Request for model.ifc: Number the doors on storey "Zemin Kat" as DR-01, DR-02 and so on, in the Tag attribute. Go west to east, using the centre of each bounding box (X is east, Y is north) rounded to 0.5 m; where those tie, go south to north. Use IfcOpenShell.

First a look at what the model holds.

```python
import ifcopenshell
import ifcopenshell.util.element
import ifcopenshell.util.placement

model = ifcopenshell.open("model.ifc")
print(model.schema)
storey = next(s for s in model.by_type("IfcBuildingStorey") if s.Name == "Zemin Kat")
doors = [e for e in ifcopenshell.util.element.get_decomposition(storey) if e.is_a("IfcDoor")]
for e in sorted(doors, key=lambda e: e.id()):
    origin = ifcopenshell.util.placement.get_local_placement(e.ObjectPlacement)[:3, 3]
    print(e.id(), e.Tag, e.Name, origin.round(2) + 0.0, sep=" | ")
```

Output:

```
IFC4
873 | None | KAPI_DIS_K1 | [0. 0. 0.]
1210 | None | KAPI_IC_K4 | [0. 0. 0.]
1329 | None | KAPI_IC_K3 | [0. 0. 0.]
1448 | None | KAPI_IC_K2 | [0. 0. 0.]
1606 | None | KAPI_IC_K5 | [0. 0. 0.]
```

```python
import ifcopenshell
import ifcopenshell.geom
import ifcopenshell.util.element
import ifcopenshell.util.shape

model = ifcopenshell.open("model.ifc")
settings = ifcopenshell.geom.settings()
settings.set("use-world-coords", True)


def centre(element):
    shape = ifcopenshell.geom.create_shape(settings, element)
    return ifcopenshell.util.shape.get_bbox_centroid(shape.geometry)


storey = next(s for s in model.by_type("IfcBuildingStorey") if s.Name == "Zemin Kat")
doors = [e for e in ifcopenshell.util.element.get_decomposition(storey) if e.is_a("IfcDoor")]

# Insertion points can sit at a corner or the storey origin, so sort by the geometry (in metres).
centres = {e: centre(e) for e in doors}
doors.sort(key=lambda e: (round(centres[e][0] / 0.5), centres[e][1]))

for i, e in enumerate(doors, start=1):
    number = f"DR-{i:02d}"
    e.Tag = number
    print(e.id(), number)

model.write("model_updated.ifc")
```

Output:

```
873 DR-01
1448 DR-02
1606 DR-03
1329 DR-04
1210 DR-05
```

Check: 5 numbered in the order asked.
